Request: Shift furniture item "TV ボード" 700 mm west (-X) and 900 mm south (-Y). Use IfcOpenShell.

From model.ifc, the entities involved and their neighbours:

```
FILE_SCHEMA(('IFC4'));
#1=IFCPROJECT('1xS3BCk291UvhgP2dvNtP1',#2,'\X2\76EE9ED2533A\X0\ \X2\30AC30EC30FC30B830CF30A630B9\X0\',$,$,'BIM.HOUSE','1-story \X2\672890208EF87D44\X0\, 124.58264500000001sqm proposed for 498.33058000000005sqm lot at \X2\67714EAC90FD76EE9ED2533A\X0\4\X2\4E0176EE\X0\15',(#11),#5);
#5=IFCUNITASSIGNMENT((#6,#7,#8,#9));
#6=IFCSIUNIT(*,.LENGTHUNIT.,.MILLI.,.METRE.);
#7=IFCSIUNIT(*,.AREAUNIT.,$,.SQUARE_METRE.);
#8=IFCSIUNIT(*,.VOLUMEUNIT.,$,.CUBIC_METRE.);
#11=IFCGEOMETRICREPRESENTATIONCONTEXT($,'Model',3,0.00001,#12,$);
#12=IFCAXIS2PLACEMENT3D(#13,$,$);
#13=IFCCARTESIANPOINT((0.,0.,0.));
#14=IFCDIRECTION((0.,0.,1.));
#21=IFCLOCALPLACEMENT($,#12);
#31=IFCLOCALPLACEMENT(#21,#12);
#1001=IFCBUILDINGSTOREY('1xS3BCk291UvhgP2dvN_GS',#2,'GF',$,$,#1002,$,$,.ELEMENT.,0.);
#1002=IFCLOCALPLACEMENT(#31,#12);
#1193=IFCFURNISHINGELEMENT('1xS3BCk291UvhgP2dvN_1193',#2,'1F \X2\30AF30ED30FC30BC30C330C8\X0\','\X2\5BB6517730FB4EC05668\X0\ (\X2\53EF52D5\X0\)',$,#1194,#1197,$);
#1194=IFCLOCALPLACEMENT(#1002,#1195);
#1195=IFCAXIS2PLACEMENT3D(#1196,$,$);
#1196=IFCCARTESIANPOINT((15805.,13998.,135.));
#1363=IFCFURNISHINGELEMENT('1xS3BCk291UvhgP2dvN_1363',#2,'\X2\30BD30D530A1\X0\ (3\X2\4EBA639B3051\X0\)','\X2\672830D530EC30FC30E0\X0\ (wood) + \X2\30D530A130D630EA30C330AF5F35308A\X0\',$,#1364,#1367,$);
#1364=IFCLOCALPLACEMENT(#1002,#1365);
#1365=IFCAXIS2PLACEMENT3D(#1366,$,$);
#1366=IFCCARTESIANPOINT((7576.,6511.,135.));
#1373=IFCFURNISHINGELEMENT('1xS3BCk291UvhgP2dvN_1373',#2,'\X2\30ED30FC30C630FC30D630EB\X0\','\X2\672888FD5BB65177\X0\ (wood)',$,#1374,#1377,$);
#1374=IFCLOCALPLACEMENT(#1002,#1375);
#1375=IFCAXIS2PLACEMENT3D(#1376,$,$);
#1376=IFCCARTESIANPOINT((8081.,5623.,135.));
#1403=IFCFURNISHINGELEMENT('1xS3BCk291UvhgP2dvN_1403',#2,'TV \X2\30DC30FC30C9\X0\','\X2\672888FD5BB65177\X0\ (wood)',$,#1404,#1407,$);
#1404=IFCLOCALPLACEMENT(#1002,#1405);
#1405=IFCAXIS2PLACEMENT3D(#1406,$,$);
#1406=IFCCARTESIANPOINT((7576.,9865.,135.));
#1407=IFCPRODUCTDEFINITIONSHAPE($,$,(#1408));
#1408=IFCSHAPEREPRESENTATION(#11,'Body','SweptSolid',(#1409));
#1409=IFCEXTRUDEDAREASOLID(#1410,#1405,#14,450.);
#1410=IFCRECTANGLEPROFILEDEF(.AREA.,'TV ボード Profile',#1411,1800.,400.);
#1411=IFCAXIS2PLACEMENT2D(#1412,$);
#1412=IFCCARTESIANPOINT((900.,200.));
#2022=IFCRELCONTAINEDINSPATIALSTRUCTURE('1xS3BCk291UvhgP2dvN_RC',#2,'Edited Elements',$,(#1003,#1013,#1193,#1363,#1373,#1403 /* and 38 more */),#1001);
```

```python
import ifcopenshell
import ifcopenshell.api.geometry
import ifcopenshell.util.placement

model = ifcopenshell.open("model.ifc")

item = model.by_guid("1xS3BCk291UvhgP2dvN_1403")
matrix = ifcopenshell.util.placement.get_local_placement(item.ObjectPlacement)
matrix[0, 3] -= 700.0
matrix[1, 3] -= 900.0
ifcopenshell.api.geometry.edit_object_placement(model, product=item, matrix=matrix, is_si=False)

print(ifcopenshell.util.placement.get_local_placement(item.ObjectPlacement).round(3) + 0.0)

model.write("model_rev.ifc")
```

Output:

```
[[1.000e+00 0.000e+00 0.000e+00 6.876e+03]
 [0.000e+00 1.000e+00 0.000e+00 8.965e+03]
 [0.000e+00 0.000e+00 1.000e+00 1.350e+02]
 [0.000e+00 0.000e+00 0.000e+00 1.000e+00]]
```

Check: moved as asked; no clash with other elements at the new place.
